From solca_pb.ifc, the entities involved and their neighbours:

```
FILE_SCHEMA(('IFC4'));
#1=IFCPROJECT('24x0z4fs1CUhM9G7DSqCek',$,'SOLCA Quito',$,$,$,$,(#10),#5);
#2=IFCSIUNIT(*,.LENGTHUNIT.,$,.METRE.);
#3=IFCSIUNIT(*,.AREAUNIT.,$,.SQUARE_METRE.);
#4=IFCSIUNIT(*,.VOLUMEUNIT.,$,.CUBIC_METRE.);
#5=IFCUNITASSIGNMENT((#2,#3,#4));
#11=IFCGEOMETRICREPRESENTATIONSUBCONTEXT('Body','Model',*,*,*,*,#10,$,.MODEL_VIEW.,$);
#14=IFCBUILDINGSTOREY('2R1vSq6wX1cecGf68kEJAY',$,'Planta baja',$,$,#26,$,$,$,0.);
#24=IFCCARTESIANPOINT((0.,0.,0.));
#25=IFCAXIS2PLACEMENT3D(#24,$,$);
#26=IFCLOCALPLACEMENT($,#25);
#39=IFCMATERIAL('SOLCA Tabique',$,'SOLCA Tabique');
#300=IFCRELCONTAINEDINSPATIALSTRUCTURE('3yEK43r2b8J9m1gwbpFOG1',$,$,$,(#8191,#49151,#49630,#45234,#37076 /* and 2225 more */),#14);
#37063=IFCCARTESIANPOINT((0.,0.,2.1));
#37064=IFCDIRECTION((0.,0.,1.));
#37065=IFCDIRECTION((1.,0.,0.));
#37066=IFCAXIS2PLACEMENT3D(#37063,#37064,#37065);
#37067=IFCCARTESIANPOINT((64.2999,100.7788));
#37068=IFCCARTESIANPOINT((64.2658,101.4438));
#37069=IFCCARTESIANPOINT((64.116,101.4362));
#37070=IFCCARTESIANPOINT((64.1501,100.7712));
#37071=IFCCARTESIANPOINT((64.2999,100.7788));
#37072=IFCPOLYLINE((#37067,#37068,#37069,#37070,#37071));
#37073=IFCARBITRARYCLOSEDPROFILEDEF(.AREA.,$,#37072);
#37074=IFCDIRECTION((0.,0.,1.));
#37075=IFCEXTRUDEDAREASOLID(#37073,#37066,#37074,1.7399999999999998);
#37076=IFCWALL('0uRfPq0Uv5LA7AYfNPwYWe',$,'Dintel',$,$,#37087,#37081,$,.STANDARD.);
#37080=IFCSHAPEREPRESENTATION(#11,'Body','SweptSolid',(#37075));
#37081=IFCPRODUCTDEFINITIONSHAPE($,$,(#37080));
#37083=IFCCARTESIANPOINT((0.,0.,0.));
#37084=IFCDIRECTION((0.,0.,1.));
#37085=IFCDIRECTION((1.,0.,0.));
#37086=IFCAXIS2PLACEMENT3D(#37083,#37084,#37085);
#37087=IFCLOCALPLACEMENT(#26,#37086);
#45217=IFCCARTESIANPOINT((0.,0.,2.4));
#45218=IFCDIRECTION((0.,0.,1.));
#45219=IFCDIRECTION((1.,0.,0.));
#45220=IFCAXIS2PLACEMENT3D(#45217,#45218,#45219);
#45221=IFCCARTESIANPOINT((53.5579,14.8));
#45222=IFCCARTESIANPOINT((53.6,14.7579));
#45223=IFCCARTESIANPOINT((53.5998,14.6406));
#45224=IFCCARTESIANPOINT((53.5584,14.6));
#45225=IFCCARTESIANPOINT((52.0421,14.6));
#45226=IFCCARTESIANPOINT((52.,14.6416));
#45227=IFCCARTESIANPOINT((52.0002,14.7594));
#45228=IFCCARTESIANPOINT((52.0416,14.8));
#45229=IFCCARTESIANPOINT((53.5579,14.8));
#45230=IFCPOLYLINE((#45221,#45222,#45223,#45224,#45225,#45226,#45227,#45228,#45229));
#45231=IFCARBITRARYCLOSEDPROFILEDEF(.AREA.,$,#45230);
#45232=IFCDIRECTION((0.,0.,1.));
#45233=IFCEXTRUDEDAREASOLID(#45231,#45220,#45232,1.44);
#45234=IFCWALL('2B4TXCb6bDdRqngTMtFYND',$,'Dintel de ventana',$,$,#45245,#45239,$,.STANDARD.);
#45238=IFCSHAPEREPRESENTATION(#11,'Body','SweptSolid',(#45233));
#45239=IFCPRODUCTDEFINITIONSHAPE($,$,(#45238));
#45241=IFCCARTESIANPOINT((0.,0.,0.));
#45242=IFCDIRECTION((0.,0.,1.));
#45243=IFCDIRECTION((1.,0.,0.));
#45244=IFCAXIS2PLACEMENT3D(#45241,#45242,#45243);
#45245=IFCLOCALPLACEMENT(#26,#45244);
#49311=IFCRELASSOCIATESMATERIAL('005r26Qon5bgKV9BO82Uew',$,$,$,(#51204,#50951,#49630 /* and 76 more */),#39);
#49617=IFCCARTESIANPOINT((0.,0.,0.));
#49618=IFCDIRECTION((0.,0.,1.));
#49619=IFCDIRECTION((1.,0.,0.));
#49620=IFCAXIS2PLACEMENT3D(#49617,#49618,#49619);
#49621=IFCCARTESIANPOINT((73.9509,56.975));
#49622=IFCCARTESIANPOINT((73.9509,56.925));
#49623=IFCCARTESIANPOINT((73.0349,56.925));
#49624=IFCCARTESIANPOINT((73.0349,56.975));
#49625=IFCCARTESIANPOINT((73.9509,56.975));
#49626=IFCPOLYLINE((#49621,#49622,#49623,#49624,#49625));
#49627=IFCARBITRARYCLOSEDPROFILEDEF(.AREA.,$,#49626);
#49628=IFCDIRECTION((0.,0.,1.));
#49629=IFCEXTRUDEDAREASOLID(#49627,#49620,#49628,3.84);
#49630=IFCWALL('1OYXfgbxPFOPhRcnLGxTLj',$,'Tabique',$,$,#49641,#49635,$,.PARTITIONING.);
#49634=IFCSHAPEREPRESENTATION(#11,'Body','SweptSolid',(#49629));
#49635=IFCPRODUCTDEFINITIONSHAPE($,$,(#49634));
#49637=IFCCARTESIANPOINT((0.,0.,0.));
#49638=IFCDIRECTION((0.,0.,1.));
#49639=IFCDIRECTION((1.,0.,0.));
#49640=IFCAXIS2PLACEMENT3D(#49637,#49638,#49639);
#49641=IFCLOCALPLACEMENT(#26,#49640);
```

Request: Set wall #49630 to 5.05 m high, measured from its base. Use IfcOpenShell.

```python
import ifcopenshell
import ifcopenshell.geom
import ifcopenshell.util.representation
import ifcopenshell.util.shape

model = ifcopenshell.open("solca_pb.ifc")
settings = ifcopenshell.geom.settings()


def volume(element):
    """Net volume in cubic metres, openings subtracted."""
    shape = ifcopenshell.geom.create_shape(settings, element)
    return ifcopenshell.util.shape.get_volume(shape.geometry)


wall = model.by_id(49630)
before = volume(wall)

body = ifcopenshell.util.representation.get_representation(wall, "Model", "Body")
solid = body.Items[0]
old_height = solid.Depth
solid.Depth = 5.05
after = volume(wall)

print(f"height {old_height:g} -> {solid.Depth:g}, volume {before:.3f} -> {after:.3f} m3")

model.write("solca_pb-out.ifc")
```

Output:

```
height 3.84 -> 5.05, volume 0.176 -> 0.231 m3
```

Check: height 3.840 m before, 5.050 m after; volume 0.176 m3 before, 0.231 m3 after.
